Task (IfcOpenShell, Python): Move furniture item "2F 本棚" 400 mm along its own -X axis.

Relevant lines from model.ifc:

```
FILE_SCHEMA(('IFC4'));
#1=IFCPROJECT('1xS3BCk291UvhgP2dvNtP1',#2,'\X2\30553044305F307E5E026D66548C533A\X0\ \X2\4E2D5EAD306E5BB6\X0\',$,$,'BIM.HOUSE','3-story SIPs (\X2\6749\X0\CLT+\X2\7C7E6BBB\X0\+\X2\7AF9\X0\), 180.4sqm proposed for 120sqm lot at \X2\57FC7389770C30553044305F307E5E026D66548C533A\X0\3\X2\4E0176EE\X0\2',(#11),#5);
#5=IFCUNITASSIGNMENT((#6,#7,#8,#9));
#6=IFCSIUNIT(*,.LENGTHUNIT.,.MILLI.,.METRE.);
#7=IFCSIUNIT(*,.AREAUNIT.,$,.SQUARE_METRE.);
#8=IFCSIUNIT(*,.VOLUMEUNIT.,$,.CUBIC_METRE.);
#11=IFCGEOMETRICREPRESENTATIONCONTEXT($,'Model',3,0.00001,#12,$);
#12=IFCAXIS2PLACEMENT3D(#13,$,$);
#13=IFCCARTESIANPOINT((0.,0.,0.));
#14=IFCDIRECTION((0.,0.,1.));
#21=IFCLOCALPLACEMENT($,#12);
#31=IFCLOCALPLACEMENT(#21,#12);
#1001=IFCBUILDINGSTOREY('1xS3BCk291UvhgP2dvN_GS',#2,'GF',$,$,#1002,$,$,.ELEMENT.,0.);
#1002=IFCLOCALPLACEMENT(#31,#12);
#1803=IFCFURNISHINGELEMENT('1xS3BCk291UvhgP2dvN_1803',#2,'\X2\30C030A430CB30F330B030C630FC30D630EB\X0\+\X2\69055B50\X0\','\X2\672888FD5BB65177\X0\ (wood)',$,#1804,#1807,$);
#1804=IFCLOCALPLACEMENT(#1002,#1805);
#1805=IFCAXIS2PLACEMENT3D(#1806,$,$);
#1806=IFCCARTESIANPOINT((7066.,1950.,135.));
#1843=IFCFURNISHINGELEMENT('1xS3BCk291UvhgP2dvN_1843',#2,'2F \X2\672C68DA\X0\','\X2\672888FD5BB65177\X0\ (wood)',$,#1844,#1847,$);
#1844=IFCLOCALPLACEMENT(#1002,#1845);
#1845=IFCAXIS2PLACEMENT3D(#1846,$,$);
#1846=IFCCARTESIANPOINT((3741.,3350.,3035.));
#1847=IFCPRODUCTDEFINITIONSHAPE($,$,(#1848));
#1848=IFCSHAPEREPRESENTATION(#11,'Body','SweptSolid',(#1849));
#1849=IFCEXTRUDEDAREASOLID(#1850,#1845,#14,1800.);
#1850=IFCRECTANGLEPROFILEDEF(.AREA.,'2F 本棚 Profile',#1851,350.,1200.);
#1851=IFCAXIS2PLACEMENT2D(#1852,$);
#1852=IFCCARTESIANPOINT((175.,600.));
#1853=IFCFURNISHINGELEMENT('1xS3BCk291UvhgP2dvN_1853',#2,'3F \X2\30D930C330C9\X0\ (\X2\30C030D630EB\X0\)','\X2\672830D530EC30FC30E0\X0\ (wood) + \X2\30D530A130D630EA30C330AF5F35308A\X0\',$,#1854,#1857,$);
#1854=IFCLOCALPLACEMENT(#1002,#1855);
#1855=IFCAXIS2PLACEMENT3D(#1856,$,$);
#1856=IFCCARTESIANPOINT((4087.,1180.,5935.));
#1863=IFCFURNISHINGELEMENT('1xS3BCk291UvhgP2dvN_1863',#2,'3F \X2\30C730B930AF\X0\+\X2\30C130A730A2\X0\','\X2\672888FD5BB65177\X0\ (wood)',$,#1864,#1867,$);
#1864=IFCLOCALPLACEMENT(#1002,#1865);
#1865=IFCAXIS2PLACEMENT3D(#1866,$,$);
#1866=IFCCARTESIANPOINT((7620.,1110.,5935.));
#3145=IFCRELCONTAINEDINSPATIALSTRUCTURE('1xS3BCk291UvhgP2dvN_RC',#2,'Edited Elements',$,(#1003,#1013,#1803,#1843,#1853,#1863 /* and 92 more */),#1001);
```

```python
import ifcopenshell
import ifcopenshell.api.geometry
import ifcopenshell.util.placement

model = ifcopenshell.open("model.ifc")

item = model.by_guid("1xS3BCk291UvhgP2dvN_1843")
matrix = ifcopenshell.util.placement.get_local_placement(item.ObjectPlacement)
matrix[:3, 3] -= matrix[:3, 0] * 400.0
ifcopenshell.api.geometry.edit_object_placement(model, product=item, matrix=matrix, is_si=False)

print(ifcopenshell.util.placement.get_local_placement(item.ObjectPlacement).round(3) + 0.0)

model.write("model_updated.ifc")
```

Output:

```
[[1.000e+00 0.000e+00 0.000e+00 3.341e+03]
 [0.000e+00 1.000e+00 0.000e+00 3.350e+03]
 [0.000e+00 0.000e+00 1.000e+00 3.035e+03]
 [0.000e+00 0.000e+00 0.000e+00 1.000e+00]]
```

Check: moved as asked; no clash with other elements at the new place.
